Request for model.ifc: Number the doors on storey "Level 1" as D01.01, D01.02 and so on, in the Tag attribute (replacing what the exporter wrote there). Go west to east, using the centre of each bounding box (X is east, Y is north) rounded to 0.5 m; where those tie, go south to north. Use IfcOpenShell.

First a look at what the model holds.

```python
import ifcopenshell
import ifcopenshell.util.element
import ifcopenshell.util.placement

model = ifcopenshell.open("model.ifc")
print(model.schema)
storey = next(s for s in model.by_type("IfcBuildingStorey") if s.Name == "Level 1")
doors = [e for e in ifcopenshell.util.element.get_decomposition(storey) if e.is_a("IfcDoor")]
for e in sorted(doors, key=lambda e: e.id()):
    origin = ifcopenshell.util.placement.get_local_placement(e.ObjectPlacement)[:3, 3]
    print(e.id(), e.Tag, e.Name, origin.round(2) + 0.0, sep=" | ")
```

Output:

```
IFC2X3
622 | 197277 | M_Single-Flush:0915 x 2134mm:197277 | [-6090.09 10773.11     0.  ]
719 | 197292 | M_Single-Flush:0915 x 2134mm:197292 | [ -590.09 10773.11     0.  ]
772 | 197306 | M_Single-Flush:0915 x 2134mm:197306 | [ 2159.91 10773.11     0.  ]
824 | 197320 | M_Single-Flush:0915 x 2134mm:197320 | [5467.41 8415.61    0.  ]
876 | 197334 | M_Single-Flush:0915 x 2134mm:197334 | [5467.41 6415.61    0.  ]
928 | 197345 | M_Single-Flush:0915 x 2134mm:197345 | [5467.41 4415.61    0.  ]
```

```python
import ifcopenshell
import ifcopenshell.geom
import ifcopenshell.util.element
import ifcopenshell.util.shape

model = ifcopenshell.open("model.ifc")
settings = ifcopenshell.geom.settings()
settings.set("use-world-coords", True)


def centre(element):
    shape = ifcopenshell.geom.create_shape(settings, element)
    return ifcopenshell.util.shape.get_bbox_centroid(shape.geometry)


storey = next(s for s in model.by_type("IfcBuildingStorey") if s.Name == "Level 1")
doors = [e for e in ifcopenshell.util.element.get_decomposition(storey) if e.is_a("IfcDoor")]

# Insertion points can sit at a corner or the storey origin, so sort by the geometry (in metres).
centres = {e: centre(e) for e in doors}
doors.sort(key=lambda e: (round(centres[e][0] / 0.5), centres[e][1]))

for i, e in enumerate(doors, start=1):
    number = f"D01.{i:02d}"
    e.Tag = number
    print(e.id(), number)

model.write("model_rev.ifc")
```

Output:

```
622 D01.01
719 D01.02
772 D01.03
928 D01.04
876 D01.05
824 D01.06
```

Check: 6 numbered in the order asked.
